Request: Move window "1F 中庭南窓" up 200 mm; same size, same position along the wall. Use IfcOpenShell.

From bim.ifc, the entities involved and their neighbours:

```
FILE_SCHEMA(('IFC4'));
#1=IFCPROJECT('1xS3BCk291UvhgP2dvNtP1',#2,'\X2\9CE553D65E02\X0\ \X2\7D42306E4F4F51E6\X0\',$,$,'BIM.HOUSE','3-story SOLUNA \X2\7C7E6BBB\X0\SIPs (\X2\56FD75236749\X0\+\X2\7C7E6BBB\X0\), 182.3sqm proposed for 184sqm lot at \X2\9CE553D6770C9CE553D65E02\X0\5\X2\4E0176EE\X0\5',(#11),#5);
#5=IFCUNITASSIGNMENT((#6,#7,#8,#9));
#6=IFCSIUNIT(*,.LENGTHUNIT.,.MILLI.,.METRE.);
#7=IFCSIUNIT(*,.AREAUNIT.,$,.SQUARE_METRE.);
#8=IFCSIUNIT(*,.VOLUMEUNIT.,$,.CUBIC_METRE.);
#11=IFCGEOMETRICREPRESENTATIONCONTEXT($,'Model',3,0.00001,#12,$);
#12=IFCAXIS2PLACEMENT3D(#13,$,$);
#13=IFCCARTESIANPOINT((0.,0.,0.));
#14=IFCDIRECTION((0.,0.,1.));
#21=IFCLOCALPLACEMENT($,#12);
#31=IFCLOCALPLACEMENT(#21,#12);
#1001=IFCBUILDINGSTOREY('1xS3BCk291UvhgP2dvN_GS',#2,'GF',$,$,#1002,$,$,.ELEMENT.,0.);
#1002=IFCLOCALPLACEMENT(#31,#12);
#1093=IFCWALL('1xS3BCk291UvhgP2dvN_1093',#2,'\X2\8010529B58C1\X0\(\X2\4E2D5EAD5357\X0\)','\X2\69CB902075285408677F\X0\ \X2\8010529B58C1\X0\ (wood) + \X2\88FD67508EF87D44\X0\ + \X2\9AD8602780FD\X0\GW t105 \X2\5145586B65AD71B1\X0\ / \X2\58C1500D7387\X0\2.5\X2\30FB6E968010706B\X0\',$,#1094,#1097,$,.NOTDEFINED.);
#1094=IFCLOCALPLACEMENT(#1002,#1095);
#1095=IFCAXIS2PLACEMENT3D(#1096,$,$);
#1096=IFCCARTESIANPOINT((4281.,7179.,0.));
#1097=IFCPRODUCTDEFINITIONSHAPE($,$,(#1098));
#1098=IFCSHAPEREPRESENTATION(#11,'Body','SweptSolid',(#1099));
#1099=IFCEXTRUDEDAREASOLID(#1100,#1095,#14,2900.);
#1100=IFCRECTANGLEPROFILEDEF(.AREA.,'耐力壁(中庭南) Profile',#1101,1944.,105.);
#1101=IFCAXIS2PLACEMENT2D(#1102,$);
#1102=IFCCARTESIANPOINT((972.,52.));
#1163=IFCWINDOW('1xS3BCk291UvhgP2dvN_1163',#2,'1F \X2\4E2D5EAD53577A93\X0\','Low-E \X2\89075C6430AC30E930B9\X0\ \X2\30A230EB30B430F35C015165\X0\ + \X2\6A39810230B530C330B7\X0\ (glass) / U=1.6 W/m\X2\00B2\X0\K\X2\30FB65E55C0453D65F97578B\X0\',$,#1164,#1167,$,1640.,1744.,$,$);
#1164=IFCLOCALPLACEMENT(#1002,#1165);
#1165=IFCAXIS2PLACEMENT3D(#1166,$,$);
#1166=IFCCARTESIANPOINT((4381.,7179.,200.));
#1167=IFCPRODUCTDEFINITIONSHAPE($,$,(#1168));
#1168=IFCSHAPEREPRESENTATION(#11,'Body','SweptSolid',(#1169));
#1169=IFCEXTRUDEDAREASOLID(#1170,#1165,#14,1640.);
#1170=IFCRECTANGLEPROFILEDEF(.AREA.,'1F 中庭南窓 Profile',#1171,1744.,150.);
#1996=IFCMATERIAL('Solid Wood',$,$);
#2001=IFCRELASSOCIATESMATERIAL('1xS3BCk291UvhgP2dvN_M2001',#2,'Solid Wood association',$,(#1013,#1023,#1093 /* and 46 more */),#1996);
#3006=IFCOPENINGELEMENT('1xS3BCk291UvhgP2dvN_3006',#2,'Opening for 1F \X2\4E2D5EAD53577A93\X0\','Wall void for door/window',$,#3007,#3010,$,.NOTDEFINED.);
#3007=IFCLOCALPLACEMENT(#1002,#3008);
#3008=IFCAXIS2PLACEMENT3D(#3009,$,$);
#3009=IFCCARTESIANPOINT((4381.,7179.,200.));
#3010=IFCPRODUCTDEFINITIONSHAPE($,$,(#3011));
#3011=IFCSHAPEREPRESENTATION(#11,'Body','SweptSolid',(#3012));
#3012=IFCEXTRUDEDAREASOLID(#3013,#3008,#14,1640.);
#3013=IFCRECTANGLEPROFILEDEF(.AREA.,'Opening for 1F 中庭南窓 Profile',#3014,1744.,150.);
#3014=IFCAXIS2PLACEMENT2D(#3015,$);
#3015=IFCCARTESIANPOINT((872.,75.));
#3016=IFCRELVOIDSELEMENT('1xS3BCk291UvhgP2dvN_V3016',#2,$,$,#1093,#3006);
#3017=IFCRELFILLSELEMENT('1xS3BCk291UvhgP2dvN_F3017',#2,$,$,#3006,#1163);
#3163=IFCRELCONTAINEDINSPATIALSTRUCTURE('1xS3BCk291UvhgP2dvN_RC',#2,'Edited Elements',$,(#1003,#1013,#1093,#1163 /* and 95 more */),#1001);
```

```python
import numpy as np
import ifcopenshell
import ifcopenshell.api.geometry
import ifcopenshell.util.placement
import ifcopenshell.util.unit

model = ifcopenshell.open("bim.ifc")
unit_scale = ifcopenshell.util.unit.calculate_unit_scale(model)

window = model.by_id(1163)
opening = window.FillsVoids[0].RelatingOpeningElement
dz = 200.0

shift = np.array([0.0, 0.0, dz])
# The window is not placed relative to its opening, so move both.
for product in (opening, window):
    matrix = ifcopenshell.util.placement.get_local_placement(product.ObjectPlacement)
    matrix[:3, 3] += shift
    ifcopenshell.api.geometry.edit_object_placement(model, product=product, matrix=matrix, is_si=False)

print(f"moved by {dz * unit_scale:+.3f} m")

model.write("bim_rev.ifc")
```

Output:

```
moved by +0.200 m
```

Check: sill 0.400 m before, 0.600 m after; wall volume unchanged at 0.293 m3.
